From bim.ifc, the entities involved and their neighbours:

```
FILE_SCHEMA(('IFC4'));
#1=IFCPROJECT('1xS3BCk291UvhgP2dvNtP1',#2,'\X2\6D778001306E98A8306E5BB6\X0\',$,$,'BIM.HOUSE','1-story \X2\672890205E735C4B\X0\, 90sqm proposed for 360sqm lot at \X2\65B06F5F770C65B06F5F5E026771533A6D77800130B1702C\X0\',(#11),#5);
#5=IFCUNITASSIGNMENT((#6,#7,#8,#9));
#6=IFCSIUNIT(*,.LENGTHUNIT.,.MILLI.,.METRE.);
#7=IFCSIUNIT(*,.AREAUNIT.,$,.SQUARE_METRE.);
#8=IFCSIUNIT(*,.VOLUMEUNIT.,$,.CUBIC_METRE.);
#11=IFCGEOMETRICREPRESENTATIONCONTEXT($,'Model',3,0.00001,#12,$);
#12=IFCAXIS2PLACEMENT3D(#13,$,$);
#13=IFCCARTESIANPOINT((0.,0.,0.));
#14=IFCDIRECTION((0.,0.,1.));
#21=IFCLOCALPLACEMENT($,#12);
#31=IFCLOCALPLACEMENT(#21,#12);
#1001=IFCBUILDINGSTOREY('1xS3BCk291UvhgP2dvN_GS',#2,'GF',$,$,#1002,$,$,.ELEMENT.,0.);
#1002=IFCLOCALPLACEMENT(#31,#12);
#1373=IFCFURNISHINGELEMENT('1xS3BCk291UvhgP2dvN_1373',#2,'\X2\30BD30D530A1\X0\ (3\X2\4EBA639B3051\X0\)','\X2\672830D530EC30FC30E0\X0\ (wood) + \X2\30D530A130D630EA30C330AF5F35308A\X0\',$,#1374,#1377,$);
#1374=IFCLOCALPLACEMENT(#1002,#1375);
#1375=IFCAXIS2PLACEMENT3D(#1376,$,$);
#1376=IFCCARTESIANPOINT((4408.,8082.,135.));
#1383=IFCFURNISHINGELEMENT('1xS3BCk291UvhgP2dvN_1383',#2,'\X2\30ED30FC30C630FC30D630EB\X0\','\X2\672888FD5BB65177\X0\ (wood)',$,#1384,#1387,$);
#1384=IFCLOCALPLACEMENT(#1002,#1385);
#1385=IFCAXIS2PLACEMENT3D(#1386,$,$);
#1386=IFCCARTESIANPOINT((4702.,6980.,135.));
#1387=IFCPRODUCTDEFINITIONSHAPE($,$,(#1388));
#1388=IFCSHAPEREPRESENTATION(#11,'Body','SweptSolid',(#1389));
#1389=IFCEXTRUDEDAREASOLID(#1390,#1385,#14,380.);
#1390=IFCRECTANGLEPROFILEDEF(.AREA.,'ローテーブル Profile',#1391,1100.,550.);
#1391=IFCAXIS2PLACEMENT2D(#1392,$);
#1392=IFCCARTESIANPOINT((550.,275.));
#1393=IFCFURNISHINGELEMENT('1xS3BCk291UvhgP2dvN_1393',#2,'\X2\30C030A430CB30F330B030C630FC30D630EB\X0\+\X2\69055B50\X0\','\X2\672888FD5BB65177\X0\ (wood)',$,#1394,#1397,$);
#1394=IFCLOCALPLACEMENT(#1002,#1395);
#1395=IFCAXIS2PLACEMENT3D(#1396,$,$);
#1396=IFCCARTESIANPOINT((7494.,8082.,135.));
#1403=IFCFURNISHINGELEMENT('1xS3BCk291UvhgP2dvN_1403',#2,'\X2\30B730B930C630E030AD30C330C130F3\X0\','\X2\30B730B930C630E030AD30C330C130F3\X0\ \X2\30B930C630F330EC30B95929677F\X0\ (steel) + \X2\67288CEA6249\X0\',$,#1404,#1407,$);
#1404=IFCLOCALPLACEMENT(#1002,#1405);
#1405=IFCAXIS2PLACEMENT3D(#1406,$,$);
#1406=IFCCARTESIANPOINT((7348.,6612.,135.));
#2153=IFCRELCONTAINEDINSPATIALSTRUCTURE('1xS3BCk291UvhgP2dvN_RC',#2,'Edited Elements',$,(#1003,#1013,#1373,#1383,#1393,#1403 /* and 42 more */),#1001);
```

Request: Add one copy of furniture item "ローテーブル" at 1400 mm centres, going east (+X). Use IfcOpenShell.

```python
import numpy as np
import ifcopenshell
import ifcopenshell.api.geometry
import ifcopenshell.api.root
import ifcopenshell.util.element
import ifcopenshell.util.placement
import ifcopenshell.util.unit

model = ifcopenshell.open("bim.ifc")
unit_scale = ifcopenshell.util.unit.calculate_unit_scale(model)


def reuse_history(source, copy):
    """copy_class also copies each property set's owner history, people and application; keep the originals."""
    for rel in copy.IsDefinedBy:
        if rel.is_a("IfcRelDefinesByProperties") and (history := rel.RelatingPropertyDefinition.OwnerHistory):
            rel.RelatingPropertyDefinition.OwnerHistory = source.OwnerHistory
            ifcopenshell.util.element.remove_deep2(model, history)


source = model.by_id(1383)
base = ifcopenshell.util.placement.get_local_placement(source.ObjectPlacement)
step = np.array([1.0, 0.0, 0.0]) * 1.4 / unit_scale

for i in range(1, 2):
    copy = ifcopenshell.api.root.copy_class(model, product=source)
    copy.Representation = ifcopenshell.util.element.copy_deep(
        model, source.Representation, exclude=["IfcGeometricRepresentationContext", "IfcRepresentationMap"]
    )
    reuse_history(source, copy)
    matrix = base.copy()
    matrix[:3, 3] += i * step
    print("added at", matrix[:3, 3].round(3) + 0.0)
    ifcopenshell.api.geometry.edit_object_placement(model, product=copy, matrix=matrix, is_si=False)

model.write("bim_edited.ifc")
```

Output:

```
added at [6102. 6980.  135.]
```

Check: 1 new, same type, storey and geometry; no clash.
